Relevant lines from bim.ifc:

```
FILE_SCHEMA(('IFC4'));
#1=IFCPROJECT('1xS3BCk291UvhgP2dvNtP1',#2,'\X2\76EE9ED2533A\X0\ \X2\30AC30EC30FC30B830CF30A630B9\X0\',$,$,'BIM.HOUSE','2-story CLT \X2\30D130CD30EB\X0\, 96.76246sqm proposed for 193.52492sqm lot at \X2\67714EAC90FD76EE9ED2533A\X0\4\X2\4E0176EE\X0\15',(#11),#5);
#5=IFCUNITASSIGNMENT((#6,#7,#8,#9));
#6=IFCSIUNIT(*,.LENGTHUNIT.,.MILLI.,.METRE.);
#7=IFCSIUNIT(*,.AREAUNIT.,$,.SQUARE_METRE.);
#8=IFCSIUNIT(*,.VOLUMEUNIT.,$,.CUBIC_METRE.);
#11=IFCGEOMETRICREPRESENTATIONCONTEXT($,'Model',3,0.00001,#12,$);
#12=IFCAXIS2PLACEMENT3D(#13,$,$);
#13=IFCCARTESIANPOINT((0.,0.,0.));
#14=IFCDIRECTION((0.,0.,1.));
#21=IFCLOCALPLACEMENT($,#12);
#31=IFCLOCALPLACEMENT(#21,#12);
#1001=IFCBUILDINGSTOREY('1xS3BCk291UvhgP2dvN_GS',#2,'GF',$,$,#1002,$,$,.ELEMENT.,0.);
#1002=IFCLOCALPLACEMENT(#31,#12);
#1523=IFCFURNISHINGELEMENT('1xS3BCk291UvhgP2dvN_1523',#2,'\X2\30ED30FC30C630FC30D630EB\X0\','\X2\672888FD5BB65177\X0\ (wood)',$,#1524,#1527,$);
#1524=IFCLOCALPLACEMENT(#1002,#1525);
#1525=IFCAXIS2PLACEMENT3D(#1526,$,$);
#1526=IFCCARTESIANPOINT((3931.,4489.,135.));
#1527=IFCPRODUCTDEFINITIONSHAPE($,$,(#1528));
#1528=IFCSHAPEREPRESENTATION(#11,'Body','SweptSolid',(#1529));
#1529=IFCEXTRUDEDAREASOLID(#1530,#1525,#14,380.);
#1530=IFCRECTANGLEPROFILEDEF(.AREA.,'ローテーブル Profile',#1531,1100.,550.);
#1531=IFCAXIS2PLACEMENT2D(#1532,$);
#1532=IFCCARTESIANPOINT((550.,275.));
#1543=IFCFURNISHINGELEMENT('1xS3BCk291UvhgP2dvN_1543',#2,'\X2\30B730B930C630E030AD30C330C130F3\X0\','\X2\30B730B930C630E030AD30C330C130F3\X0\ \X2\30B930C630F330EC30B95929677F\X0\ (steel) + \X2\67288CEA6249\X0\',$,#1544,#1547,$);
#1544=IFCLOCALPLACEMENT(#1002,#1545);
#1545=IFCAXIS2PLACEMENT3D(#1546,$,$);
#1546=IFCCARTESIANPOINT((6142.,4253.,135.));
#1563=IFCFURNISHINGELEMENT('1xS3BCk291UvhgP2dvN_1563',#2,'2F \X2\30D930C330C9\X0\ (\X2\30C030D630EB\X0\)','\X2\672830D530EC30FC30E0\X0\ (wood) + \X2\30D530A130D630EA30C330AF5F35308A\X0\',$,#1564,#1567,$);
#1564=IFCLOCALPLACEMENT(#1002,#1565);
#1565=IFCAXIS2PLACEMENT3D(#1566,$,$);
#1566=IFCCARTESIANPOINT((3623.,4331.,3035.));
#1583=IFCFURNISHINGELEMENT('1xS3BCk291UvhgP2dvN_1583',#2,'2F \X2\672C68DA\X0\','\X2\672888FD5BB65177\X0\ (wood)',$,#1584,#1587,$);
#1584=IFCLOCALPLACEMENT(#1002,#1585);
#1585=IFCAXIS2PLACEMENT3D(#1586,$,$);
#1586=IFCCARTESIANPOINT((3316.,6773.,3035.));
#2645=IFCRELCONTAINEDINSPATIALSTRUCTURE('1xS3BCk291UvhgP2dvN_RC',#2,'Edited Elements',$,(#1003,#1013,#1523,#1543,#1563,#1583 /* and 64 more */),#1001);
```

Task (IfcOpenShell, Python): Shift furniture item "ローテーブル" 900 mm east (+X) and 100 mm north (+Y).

```python
import ifcopenshell
import ifcopenshell.api.geometry
import ifcopenshell.util.placement
import ifcopenshell.util.unit

model = ifcopenshell.open("bim.ifc")
unit_scale = ifcopenshell.util.unit.calculate_unit_scale(model)

item = model.by_id(1523)
matrix = ifcopenshell.util.placement.get_local_placement(item.ObjectPlacement)
matrix[0, 3] += 0.9 / unit_scale
matrix[1, 3] += 0.1 / unit_scale
ifcopenshell.api.geometry.edit_object_placement(model, product=item, matrix=matrix, is_si=False)

print(ifcopenshell.util.placement.get_local_placement(item.ObjectPlacement).round(3) + 0.0)

model.write("bim-out.ifc")
```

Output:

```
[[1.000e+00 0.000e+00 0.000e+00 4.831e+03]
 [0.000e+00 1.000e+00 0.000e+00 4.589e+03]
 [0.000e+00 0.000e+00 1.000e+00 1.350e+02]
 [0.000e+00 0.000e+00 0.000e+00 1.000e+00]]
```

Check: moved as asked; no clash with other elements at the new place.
